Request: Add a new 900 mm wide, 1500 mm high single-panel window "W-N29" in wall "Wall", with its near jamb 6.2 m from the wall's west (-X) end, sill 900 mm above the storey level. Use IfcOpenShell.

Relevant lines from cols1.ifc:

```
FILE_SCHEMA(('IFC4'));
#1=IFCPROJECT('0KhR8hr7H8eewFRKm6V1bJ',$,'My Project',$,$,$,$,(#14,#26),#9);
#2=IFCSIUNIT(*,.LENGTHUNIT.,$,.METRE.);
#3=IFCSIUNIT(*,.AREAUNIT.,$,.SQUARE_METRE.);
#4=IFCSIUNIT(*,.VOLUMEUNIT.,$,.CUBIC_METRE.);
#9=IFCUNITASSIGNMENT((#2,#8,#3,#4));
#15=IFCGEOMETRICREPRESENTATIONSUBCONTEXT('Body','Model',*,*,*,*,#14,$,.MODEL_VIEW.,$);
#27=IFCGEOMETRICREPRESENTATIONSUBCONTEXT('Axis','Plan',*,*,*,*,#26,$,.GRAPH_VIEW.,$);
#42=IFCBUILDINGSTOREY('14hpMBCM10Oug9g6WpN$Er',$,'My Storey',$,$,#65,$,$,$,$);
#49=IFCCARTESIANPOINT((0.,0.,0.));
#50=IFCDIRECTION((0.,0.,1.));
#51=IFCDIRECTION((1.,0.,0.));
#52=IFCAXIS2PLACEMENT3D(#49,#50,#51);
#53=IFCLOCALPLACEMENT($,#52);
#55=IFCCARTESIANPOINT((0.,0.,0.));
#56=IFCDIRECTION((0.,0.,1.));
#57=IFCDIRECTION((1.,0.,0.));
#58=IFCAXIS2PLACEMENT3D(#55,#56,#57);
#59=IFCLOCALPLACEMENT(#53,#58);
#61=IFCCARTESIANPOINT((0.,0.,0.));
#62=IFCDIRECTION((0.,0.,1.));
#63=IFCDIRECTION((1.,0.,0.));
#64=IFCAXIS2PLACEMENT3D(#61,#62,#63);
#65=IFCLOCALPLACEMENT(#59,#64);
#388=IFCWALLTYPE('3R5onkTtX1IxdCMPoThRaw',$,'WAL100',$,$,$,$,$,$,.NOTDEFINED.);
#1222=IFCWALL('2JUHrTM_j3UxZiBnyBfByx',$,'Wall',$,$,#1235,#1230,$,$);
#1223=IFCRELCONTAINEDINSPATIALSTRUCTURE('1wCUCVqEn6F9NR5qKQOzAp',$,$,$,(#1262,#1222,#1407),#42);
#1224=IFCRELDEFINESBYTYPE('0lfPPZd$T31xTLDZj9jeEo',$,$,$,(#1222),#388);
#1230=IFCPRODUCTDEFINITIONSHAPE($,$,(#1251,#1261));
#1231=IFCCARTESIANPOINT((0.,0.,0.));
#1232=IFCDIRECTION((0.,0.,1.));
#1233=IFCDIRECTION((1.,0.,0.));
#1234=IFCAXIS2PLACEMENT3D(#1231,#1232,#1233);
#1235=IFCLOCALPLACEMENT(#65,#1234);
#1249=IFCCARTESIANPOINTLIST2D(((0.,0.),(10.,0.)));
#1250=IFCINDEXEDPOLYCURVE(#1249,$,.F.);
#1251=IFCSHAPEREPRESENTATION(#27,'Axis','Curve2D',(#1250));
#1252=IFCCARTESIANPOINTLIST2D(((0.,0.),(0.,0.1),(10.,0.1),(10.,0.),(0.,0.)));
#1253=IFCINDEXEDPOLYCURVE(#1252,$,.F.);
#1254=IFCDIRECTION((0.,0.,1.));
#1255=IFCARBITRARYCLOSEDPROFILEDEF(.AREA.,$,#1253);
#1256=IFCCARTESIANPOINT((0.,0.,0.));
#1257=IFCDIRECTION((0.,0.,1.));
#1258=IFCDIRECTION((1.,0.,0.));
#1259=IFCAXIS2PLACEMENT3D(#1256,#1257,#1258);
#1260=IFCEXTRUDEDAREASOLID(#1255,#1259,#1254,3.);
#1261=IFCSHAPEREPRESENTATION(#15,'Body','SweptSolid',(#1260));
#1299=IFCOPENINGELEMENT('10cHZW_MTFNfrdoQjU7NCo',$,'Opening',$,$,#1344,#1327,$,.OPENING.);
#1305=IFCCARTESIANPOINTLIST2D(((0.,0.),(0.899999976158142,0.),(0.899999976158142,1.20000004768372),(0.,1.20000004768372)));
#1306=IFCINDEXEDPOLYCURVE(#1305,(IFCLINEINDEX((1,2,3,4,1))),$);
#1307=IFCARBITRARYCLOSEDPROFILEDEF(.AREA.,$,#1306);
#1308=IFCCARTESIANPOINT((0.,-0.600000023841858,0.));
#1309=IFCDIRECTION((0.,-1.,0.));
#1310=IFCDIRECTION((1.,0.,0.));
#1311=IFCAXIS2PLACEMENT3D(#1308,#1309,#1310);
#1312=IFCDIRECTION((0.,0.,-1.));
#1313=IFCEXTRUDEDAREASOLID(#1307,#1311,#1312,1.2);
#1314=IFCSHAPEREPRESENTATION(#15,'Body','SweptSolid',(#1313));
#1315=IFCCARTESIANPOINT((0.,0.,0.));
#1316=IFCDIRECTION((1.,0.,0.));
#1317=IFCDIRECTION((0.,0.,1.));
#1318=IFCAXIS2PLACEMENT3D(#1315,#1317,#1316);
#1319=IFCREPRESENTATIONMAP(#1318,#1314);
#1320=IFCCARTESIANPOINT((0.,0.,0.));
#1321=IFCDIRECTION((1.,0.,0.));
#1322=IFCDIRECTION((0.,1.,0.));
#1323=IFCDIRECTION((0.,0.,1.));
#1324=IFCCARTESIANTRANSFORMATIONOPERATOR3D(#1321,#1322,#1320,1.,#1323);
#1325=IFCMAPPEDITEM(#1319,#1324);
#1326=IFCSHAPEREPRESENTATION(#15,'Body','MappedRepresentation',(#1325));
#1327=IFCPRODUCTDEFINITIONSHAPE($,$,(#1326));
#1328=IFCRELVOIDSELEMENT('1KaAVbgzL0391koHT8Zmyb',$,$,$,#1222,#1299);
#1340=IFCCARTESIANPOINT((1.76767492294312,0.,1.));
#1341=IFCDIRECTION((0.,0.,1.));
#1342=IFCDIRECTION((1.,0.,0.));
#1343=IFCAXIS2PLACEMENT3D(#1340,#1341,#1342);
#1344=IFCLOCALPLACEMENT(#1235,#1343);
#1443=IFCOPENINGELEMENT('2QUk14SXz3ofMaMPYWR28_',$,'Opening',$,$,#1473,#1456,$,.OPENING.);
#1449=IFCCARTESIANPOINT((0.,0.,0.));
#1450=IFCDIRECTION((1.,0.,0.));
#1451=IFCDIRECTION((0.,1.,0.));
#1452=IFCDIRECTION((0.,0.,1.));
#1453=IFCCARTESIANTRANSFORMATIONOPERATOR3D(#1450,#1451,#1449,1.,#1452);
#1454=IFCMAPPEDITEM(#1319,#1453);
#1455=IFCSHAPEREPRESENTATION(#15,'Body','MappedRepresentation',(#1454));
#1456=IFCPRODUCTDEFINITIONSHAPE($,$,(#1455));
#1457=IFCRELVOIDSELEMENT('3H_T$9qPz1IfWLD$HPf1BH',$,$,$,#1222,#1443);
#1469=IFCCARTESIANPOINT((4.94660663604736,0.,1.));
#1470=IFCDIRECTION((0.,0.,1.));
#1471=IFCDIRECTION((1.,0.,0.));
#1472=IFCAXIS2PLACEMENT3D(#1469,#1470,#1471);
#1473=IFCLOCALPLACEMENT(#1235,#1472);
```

```python
import numpy as np
import ifcopenshell
import ifcopenshell.api.feature
import ifcopenshell.api.geometry
import ifcopenshell.api.root
import ifcopenshell.api.spatial
import ifcopenshell.geom
import ifcopenshell.util.element
import ifcopenshell.util.placement
import ifcopenshell.util.representation
import ifcopenshell.util.shape
import ifcopenshell.util.unit

model = ifcopenshell.open("cols1.ifc")
unit_scale = ifcopenshell.util.unit.calculate_unit_scale(model)
settings = ifcopenshell.geom.settings()


def volume(element):
    """Net volume in cubic metres, openings subtracted."""
    shape = ifcopenshell.geom.create_shape(settings, element)
    return ifcopenshell.util.shape.get_volume(shape.geometry)


wall = model.by_guid("2JUHrTM_j3UxZiBnyBfByx")
storey = ifcopenshell.util.element.get_container(wall, ifc_class="IfcBuildingStorey")
context = ifcopenshell.util.representation.get_context(model, "Model", "Body", "MODEL_VIEW")
before = volume(wall)

width, height, from_end, sill = 0.9, 1.5, 6.2, 0.9  # metres

# The wall runs along its own X axis, and the end named is its -X end.
wall_shape = ifcopenshell.geom.create_shape(settings, wall)
x, y, z = ifcopenshell.util.shape.get_vertices(wall_shape.geometry).T
start = x.min() + from_end
face, thickness = float(y.min()), float(y.max() - y.min())
wall_matrix = ifcopenshell.util.placement.get_local_placement(wall.ObjectPlacement)
level = ifcopenshell.util.placement.get_local_placement(storey.ObjectPlacement)[2, 3]


def in_wall(x, y):
    """Placement at x, y metres in the wall's axes, at sill height."""
    matrix = wall_matrix.copy()
    matrix[:, 3] = wall_matrix @ np.array([x / unit_scale, y / unit_scale, 0.0, 1.0])
    matrix[2, 3] = level + sill / unit_scale
    return matrix


# Opening: a box that overshoots both wall faces by 50 mm.
opening = ifcopenshell.api.root.create_entity(model, ifc_class="IfcOpeningElement", predefined_type="OPENING")
box = ifcopenshell.api.geometry.add_wall_representation(
    model, context=context, length=width, height=height, thickness=thickness + 0.1
)
ifcopenshell.api.geometry.assign_representation(model, product=opening, representation=box)
ifcopenshell.api.geometry.edit_object_placement(model, product=opening, matrix=in_wall(start, face - 0.05), is_si=False)
ifcopenshell.api.feature.add_feature(model, feature=opening, element=wall)

window = ifcopenshell.api.root.create_entity(model, ifc_class="IfcWindow", name="W-N29", predefined_type="WINDOW")
window.OverallWidth, window.OverallHeight = width / unit_scale, height / unit_scale
window.PartitioningType = "SINGLE_PANEL"
body = ifcopenshell.api.geometry.add_window_representation(
    model,
    context=context,
    overall_width=window.OverallWidth,
    overall_height=window.OverallHeight,
    partition_type="SINGLE_PANEL",
)
ifcopenshell.api.geometry.assign_representation(model, product=window, representation=body)
ifcopenshell.api.spatial.assign_container(model, products=[window], relating_structure=storey)
ifcopenshell.api.feature.add_filling(model, opening=opening, element=window)

# Centre the window in the wall's thickness.
ifcopenshell.api.geometry.edit_object_placement(model, product=window, matrix=in_wall(start, face), is_si=False)
window_shape = ifcopenshell.geom.create_shape(settings, window)
depth = ifcopenshell.util.shape.get_vertices(window_shape.geometry)[:, 1]
offset = face + thickness / 2 - (depth.min() + depth.max()) / 2
ifcopenshell.api.geometry.edit_object_placement(model, product=window, matrix=in_wall(start, offset), is_si=False)

after = volume(wall)

print(f"wall volume {before:.3f} -> {after:.3f} m3")

model.write("cols1_edited.ifc")
```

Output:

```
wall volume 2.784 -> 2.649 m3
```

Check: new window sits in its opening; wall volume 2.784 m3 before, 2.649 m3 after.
